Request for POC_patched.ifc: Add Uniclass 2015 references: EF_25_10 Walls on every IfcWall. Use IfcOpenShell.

First a look at what the model holds.

```python
import ifcopenshell

model = ifcopenshell.open("POC_patched.ifc")
print(model.schema)
print("classifications:", [c.Name for c in model.by_type("IfcClassification")])
for ifc_class in ("IfcDoor", "IfcRoof", "IfcStair", "IfcWall", "IfcWindow"):
    print(ifc_class, len(model.by_type(ifc_class)))
```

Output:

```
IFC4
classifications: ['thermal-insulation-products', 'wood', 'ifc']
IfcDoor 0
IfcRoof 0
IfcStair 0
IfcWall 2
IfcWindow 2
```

```python
import ifcopenshell
import ifcopenshell.api.classification

model = ifcopenshell.open("POC_patched.ifc")

system = ifcopenshell.api.classification.add_classification(model, classification="Uniclass 2015")

codes = {
    "IfcWall": ("EF_25_10", "Walls"),
}
for ifc_class, (code, name) in codes.items():
    products = model.by_type(ifc_class)
    ifcopenshell.api.classification.add_reference(
        model, products=products, classification=system, identification=code, name=name
    )
    print(code, len(products))

model.write("POC_patched_edited.ifc")
```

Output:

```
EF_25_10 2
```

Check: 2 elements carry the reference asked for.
